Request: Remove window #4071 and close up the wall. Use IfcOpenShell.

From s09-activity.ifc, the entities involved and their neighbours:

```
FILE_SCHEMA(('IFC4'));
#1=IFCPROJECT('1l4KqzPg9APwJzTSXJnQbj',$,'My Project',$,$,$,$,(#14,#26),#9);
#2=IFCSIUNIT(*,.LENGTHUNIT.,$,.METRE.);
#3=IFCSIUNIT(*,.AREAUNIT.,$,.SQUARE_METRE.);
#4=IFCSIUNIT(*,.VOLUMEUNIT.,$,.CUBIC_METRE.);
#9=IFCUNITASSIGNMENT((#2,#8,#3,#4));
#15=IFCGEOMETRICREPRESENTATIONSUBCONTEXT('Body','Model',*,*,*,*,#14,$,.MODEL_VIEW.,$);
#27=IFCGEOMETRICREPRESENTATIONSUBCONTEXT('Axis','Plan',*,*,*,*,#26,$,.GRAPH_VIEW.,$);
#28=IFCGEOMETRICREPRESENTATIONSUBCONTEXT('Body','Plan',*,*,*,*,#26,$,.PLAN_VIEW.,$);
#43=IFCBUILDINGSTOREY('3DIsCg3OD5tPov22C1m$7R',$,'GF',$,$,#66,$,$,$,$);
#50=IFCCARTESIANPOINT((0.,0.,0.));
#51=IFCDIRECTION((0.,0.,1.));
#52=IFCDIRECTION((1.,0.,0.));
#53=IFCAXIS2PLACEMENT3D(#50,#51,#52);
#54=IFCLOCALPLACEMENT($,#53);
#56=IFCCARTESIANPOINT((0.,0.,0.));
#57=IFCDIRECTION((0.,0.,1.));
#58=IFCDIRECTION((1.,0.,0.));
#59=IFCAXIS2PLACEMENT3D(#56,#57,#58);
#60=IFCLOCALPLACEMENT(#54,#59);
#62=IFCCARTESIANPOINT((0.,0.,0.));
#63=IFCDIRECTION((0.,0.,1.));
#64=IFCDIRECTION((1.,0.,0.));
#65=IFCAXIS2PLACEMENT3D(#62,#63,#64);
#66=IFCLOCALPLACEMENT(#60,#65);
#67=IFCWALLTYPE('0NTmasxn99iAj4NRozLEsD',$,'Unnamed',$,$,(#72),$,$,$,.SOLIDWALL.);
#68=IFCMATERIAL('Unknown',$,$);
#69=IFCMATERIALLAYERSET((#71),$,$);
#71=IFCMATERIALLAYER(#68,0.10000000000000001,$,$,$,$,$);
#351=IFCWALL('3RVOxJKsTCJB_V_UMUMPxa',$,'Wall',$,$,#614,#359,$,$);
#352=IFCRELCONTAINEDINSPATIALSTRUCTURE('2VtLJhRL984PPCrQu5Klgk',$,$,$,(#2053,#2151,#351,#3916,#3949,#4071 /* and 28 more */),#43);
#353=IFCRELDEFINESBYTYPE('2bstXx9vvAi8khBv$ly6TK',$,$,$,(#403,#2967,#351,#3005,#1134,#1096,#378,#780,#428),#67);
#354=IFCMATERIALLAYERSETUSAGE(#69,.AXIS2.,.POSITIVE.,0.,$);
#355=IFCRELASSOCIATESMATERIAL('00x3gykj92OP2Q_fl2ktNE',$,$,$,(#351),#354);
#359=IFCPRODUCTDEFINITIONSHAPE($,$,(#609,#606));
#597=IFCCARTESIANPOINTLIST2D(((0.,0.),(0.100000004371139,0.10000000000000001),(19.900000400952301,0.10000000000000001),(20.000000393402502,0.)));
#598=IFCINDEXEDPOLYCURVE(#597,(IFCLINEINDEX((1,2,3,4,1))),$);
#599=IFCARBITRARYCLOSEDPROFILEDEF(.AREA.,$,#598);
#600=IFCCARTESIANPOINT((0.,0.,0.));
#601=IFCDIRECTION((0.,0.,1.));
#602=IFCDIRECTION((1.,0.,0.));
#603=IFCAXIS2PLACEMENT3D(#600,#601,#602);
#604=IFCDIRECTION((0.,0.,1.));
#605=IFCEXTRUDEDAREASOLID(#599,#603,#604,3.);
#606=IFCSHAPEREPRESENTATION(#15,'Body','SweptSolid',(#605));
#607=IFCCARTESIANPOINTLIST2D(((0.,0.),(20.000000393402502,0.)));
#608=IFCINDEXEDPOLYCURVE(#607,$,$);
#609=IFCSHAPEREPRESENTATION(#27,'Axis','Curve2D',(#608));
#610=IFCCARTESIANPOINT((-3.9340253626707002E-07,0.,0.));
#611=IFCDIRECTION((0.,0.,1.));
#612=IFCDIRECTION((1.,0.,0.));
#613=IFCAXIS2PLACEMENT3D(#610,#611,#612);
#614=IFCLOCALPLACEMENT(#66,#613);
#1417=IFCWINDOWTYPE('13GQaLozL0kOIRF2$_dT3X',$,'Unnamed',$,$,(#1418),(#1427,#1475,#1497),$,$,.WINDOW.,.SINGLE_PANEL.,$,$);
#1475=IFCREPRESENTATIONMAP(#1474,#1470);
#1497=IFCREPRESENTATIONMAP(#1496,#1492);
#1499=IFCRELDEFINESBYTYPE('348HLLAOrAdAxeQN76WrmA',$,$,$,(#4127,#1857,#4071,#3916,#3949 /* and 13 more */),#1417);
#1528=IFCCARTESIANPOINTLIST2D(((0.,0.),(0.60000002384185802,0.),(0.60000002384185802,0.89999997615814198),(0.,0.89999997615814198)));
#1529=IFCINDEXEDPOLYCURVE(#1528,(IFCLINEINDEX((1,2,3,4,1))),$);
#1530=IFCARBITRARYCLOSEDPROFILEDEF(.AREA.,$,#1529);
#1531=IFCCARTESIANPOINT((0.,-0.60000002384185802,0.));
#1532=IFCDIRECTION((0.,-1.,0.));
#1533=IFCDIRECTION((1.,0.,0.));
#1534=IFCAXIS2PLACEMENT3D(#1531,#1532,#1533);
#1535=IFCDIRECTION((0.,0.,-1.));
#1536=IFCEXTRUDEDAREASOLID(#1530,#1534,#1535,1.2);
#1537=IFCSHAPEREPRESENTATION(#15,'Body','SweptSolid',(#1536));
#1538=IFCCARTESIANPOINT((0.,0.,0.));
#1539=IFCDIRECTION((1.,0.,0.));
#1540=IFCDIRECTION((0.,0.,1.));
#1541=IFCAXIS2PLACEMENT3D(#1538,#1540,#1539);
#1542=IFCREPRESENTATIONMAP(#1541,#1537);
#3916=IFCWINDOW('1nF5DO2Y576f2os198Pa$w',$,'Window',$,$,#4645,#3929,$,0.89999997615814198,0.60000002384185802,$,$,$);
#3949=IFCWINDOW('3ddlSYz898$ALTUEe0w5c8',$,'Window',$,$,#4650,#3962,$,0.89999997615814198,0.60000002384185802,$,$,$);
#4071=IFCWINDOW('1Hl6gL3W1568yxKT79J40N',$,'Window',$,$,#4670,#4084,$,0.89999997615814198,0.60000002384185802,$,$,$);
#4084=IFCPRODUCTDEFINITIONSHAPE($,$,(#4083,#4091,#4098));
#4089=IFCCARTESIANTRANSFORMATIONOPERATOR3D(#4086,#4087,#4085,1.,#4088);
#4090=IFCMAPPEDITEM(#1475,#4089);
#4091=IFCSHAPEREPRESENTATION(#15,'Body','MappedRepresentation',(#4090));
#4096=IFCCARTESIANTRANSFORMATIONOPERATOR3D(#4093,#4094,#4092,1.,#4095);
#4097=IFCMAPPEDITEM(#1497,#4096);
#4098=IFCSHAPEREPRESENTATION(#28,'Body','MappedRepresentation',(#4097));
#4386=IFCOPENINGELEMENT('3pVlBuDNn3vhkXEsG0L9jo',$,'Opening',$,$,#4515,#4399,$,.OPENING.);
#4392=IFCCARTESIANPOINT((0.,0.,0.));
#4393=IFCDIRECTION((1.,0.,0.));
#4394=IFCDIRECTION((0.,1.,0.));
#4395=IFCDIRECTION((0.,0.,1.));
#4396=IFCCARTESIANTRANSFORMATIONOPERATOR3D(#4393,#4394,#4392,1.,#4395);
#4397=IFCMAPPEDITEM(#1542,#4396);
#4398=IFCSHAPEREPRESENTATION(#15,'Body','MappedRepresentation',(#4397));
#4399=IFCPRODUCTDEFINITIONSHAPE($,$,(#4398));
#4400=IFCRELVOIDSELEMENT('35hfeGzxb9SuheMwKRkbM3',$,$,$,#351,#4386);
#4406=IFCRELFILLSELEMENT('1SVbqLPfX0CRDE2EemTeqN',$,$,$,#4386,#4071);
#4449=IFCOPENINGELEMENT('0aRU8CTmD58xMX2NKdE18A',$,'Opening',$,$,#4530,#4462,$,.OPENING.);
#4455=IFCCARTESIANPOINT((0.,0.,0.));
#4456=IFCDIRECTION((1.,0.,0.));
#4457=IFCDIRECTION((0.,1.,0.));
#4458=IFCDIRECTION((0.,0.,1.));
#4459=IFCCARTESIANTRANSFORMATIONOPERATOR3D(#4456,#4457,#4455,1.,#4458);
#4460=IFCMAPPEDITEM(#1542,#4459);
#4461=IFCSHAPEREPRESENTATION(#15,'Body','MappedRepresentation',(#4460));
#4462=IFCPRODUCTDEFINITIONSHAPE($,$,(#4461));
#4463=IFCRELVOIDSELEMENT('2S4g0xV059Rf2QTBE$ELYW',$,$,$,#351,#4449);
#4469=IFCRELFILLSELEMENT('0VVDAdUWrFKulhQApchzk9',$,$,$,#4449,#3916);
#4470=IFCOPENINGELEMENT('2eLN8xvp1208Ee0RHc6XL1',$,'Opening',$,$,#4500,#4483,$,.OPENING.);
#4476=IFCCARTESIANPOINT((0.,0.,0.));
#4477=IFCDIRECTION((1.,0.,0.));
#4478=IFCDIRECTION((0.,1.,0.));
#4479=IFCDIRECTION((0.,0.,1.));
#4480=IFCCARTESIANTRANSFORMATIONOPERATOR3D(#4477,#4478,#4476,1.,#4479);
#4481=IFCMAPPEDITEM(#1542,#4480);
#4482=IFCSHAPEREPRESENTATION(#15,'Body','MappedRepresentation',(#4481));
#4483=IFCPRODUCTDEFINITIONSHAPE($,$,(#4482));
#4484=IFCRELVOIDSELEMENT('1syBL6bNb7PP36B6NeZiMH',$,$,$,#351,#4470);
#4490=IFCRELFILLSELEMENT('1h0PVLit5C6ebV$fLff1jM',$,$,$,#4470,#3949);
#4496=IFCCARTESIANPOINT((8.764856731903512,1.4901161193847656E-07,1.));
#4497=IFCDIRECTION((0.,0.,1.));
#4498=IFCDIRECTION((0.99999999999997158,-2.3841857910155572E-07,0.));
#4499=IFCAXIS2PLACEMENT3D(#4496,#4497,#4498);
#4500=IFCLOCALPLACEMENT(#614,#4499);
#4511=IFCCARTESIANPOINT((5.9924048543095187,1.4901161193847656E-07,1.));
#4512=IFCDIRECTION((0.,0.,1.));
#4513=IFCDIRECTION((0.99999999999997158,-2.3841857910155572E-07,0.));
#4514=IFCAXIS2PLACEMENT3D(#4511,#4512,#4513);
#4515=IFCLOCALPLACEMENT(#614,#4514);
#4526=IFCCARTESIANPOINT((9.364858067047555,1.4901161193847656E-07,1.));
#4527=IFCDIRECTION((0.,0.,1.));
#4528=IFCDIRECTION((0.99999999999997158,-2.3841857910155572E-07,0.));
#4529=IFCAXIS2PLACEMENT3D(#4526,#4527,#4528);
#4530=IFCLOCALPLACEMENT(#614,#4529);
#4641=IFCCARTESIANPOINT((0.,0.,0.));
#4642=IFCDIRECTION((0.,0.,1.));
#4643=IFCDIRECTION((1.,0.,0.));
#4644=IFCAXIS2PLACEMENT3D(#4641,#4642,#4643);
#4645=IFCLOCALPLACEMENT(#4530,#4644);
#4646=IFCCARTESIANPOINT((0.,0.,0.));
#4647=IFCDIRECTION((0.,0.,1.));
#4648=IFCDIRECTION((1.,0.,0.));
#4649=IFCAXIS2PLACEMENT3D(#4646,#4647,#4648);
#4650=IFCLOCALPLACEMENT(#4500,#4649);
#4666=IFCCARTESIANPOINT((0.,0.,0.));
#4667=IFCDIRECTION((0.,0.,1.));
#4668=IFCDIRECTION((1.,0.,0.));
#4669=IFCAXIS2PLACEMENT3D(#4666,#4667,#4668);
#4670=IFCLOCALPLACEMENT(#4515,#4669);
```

```python
import ifcopenshell
import ifcopenshell.api.feature
import ifcopenshell.api.root
import ifcopenshell.geom
import ifcopenshell.util.shape

model = ifcopenshell.open("s09-activity.ifc")
settings = ifcopenshell.geom.settings()


def volume(element):
    """Net volume in cubic metres, openings subtracted."""
    shape = ifcopenshell.geom.create_shape(settings, element)
    return ifcopenshell.util.shape.get_volume(shape.geometry)


window = model.by_id(4071)
opening = window.FillsVoids[0].RelatingOpeningElement
wall = opening.VoidsElements[0].RelatingBuildingElement
before = volume(wall)

ifcopenshell.api.root.remove_product(model, product=window)
ifcopenshell.api.feature.remove_feature(model, feature=opening)

after = volume(wall)

print(f"wall volume {before:.3f} -> {after:.3f} m3")

model.write("s09-activity_updated.ifc")
```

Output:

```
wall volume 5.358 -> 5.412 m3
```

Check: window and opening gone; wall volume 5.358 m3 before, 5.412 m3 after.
